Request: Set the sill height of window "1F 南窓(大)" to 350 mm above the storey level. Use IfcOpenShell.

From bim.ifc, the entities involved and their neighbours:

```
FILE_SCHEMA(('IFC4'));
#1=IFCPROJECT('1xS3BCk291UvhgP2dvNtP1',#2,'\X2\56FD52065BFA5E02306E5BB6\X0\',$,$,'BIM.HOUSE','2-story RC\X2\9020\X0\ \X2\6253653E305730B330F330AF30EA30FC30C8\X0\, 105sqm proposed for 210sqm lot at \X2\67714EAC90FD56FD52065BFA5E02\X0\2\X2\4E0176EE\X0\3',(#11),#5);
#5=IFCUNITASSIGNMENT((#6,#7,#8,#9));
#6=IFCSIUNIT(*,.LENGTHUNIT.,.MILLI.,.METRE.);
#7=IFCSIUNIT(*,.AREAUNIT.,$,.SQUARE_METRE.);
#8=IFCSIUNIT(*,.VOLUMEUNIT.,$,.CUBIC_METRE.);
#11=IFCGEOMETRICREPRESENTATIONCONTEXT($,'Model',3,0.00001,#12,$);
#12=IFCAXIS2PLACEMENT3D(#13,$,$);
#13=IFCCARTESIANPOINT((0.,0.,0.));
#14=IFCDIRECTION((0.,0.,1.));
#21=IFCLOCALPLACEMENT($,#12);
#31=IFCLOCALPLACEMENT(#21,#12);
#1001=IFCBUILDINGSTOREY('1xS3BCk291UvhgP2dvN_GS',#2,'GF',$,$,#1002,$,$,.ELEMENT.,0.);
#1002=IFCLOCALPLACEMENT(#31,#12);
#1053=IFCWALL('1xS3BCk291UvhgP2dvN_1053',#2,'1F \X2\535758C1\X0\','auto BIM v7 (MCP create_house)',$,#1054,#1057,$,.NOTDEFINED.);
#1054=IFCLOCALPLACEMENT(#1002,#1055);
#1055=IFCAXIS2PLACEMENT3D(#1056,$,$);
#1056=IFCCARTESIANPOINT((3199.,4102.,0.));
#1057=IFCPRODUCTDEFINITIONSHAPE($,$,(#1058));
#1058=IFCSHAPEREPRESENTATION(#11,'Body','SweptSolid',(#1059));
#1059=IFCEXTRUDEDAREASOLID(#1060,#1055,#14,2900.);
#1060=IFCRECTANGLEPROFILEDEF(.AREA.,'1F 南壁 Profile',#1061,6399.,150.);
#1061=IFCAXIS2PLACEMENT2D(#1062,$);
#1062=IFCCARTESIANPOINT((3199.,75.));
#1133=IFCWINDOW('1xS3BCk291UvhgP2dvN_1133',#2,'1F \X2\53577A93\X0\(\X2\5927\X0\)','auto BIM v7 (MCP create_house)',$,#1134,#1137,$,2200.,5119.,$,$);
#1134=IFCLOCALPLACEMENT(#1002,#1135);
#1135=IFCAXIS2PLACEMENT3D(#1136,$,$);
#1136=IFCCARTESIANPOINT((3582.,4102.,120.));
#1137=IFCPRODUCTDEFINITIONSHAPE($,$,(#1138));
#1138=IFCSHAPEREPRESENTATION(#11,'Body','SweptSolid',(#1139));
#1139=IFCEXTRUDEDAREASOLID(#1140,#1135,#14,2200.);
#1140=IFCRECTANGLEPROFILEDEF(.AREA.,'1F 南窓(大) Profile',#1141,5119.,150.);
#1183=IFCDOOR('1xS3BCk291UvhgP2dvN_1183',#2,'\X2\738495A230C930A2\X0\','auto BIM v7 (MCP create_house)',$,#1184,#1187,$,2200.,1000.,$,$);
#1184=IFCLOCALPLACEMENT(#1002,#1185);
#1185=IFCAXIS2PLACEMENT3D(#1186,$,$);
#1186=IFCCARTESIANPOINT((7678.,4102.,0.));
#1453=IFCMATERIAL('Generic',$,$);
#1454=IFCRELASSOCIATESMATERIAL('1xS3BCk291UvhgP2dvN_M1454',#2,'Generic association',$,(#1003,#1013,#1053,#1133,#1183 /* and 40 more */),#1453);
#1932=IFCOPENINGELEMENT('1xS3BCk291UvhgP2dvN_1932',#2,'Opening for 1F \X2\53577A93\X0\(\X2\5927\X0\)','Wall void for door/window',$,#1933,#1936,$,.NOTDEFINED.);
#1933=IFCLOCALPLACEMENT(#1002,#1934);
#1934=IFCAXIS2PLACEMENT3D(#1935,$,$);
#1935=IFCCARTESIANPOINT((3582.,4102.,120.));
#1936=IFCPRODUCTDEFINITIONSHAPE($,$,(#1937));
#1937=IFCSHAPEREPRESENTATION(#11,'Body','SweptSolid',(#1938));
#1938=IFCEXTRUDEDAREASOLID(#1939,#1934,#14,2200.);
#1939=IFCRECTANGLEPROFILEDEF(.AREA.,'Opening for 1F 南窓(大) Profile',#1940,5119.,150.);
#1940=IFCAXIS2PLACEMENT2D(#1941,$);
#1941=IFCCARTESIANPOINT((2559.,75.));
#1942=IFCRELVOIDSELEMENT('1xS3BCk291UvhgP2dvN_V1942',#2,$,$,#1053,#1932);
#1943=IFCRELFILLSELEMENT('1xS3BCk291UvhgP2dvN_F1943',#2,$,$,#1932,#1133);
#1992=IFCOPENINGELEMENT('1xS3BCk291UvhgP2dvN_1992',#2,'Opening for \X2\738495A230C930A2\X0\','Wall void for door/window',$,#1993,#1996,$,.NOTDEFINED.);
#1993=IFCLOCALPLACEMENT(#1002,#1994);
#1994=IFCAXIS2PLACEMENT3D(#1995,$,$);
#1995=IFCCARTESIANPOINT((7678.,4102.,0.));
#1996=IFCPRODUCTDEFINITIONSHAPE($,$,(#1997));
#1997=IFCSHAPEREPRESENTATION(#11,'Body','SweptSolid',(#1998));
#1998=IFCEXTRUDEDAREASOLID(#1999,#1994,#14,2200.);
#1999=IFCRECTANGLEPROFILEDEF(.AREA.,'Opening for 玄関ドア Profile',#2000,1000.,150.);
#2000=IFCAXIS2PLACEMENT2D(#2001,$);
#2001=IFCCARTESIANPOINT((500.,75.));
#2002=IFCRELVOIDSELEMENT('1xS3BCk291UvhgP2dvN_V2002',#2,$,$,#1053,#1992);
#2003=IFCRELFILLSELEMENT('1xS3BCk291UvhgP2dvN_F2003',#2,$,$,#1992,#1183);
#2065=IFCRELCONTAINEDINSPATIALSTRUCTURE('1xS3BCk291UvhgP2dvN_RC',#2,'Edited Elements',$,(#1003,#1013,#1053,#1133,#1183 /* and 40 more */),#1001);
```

```python
import numpy as np
import ifcopenshell
import ifcopenshell.api.geometry
import ifcopenshell.geom
import ifcopenshell.util.element
import ifcopenshell.util.placement
import ifcopenshell.util.shape
import ifcopenshell.util.unit

model = ifcopenshell.open("bim.ifc")
unit_scale = ifcopenshell.util.unit.calculate_unit_scale(model)

window = model.by_guid("1xS3BCk291UvhgP2dvN_1133")
opening = window.FillsVoids[0].RelatingOpeningElement
storey = ifcopenshell.util.element.get_container(window, ifc_class="IfcBuildingStorey")
level = ifcopenshell.util.placement.get_local_placement(storey.ObjectPlacement)[2, 3]

# The opening's origin need not be at the sill, so measure its lowest point.
shape = ifcopenshell.geom.create_shape(ifcopenshell.geom.settings(), opening)
bottom = ifcopenshell.util.shape.get_shape_bottom_elevation(shape, shape.geometry) / unit_scale
dz = level + 0.35 / unit_scale - bottom

shift = np.array([0.0, 0.0, dz])
# The window is not placed relative to its opening, so move both.
for product in (opening, window):
    matrix = ifcopenshell.util.placement.get_local_placement(product.ObjectPlacement)
    matrix[:3, 3] += shift
    ifcopenshell.api.geometry.edit_object_placement(model, product=product, matrix=matrix, is_si=False)

print(f"moved by {dz * unit_scale:+.3f} m")

model.write("bim-out.ifc")
```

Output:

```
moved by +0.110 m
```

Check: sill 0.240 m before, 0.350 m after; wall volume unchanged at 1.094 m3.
